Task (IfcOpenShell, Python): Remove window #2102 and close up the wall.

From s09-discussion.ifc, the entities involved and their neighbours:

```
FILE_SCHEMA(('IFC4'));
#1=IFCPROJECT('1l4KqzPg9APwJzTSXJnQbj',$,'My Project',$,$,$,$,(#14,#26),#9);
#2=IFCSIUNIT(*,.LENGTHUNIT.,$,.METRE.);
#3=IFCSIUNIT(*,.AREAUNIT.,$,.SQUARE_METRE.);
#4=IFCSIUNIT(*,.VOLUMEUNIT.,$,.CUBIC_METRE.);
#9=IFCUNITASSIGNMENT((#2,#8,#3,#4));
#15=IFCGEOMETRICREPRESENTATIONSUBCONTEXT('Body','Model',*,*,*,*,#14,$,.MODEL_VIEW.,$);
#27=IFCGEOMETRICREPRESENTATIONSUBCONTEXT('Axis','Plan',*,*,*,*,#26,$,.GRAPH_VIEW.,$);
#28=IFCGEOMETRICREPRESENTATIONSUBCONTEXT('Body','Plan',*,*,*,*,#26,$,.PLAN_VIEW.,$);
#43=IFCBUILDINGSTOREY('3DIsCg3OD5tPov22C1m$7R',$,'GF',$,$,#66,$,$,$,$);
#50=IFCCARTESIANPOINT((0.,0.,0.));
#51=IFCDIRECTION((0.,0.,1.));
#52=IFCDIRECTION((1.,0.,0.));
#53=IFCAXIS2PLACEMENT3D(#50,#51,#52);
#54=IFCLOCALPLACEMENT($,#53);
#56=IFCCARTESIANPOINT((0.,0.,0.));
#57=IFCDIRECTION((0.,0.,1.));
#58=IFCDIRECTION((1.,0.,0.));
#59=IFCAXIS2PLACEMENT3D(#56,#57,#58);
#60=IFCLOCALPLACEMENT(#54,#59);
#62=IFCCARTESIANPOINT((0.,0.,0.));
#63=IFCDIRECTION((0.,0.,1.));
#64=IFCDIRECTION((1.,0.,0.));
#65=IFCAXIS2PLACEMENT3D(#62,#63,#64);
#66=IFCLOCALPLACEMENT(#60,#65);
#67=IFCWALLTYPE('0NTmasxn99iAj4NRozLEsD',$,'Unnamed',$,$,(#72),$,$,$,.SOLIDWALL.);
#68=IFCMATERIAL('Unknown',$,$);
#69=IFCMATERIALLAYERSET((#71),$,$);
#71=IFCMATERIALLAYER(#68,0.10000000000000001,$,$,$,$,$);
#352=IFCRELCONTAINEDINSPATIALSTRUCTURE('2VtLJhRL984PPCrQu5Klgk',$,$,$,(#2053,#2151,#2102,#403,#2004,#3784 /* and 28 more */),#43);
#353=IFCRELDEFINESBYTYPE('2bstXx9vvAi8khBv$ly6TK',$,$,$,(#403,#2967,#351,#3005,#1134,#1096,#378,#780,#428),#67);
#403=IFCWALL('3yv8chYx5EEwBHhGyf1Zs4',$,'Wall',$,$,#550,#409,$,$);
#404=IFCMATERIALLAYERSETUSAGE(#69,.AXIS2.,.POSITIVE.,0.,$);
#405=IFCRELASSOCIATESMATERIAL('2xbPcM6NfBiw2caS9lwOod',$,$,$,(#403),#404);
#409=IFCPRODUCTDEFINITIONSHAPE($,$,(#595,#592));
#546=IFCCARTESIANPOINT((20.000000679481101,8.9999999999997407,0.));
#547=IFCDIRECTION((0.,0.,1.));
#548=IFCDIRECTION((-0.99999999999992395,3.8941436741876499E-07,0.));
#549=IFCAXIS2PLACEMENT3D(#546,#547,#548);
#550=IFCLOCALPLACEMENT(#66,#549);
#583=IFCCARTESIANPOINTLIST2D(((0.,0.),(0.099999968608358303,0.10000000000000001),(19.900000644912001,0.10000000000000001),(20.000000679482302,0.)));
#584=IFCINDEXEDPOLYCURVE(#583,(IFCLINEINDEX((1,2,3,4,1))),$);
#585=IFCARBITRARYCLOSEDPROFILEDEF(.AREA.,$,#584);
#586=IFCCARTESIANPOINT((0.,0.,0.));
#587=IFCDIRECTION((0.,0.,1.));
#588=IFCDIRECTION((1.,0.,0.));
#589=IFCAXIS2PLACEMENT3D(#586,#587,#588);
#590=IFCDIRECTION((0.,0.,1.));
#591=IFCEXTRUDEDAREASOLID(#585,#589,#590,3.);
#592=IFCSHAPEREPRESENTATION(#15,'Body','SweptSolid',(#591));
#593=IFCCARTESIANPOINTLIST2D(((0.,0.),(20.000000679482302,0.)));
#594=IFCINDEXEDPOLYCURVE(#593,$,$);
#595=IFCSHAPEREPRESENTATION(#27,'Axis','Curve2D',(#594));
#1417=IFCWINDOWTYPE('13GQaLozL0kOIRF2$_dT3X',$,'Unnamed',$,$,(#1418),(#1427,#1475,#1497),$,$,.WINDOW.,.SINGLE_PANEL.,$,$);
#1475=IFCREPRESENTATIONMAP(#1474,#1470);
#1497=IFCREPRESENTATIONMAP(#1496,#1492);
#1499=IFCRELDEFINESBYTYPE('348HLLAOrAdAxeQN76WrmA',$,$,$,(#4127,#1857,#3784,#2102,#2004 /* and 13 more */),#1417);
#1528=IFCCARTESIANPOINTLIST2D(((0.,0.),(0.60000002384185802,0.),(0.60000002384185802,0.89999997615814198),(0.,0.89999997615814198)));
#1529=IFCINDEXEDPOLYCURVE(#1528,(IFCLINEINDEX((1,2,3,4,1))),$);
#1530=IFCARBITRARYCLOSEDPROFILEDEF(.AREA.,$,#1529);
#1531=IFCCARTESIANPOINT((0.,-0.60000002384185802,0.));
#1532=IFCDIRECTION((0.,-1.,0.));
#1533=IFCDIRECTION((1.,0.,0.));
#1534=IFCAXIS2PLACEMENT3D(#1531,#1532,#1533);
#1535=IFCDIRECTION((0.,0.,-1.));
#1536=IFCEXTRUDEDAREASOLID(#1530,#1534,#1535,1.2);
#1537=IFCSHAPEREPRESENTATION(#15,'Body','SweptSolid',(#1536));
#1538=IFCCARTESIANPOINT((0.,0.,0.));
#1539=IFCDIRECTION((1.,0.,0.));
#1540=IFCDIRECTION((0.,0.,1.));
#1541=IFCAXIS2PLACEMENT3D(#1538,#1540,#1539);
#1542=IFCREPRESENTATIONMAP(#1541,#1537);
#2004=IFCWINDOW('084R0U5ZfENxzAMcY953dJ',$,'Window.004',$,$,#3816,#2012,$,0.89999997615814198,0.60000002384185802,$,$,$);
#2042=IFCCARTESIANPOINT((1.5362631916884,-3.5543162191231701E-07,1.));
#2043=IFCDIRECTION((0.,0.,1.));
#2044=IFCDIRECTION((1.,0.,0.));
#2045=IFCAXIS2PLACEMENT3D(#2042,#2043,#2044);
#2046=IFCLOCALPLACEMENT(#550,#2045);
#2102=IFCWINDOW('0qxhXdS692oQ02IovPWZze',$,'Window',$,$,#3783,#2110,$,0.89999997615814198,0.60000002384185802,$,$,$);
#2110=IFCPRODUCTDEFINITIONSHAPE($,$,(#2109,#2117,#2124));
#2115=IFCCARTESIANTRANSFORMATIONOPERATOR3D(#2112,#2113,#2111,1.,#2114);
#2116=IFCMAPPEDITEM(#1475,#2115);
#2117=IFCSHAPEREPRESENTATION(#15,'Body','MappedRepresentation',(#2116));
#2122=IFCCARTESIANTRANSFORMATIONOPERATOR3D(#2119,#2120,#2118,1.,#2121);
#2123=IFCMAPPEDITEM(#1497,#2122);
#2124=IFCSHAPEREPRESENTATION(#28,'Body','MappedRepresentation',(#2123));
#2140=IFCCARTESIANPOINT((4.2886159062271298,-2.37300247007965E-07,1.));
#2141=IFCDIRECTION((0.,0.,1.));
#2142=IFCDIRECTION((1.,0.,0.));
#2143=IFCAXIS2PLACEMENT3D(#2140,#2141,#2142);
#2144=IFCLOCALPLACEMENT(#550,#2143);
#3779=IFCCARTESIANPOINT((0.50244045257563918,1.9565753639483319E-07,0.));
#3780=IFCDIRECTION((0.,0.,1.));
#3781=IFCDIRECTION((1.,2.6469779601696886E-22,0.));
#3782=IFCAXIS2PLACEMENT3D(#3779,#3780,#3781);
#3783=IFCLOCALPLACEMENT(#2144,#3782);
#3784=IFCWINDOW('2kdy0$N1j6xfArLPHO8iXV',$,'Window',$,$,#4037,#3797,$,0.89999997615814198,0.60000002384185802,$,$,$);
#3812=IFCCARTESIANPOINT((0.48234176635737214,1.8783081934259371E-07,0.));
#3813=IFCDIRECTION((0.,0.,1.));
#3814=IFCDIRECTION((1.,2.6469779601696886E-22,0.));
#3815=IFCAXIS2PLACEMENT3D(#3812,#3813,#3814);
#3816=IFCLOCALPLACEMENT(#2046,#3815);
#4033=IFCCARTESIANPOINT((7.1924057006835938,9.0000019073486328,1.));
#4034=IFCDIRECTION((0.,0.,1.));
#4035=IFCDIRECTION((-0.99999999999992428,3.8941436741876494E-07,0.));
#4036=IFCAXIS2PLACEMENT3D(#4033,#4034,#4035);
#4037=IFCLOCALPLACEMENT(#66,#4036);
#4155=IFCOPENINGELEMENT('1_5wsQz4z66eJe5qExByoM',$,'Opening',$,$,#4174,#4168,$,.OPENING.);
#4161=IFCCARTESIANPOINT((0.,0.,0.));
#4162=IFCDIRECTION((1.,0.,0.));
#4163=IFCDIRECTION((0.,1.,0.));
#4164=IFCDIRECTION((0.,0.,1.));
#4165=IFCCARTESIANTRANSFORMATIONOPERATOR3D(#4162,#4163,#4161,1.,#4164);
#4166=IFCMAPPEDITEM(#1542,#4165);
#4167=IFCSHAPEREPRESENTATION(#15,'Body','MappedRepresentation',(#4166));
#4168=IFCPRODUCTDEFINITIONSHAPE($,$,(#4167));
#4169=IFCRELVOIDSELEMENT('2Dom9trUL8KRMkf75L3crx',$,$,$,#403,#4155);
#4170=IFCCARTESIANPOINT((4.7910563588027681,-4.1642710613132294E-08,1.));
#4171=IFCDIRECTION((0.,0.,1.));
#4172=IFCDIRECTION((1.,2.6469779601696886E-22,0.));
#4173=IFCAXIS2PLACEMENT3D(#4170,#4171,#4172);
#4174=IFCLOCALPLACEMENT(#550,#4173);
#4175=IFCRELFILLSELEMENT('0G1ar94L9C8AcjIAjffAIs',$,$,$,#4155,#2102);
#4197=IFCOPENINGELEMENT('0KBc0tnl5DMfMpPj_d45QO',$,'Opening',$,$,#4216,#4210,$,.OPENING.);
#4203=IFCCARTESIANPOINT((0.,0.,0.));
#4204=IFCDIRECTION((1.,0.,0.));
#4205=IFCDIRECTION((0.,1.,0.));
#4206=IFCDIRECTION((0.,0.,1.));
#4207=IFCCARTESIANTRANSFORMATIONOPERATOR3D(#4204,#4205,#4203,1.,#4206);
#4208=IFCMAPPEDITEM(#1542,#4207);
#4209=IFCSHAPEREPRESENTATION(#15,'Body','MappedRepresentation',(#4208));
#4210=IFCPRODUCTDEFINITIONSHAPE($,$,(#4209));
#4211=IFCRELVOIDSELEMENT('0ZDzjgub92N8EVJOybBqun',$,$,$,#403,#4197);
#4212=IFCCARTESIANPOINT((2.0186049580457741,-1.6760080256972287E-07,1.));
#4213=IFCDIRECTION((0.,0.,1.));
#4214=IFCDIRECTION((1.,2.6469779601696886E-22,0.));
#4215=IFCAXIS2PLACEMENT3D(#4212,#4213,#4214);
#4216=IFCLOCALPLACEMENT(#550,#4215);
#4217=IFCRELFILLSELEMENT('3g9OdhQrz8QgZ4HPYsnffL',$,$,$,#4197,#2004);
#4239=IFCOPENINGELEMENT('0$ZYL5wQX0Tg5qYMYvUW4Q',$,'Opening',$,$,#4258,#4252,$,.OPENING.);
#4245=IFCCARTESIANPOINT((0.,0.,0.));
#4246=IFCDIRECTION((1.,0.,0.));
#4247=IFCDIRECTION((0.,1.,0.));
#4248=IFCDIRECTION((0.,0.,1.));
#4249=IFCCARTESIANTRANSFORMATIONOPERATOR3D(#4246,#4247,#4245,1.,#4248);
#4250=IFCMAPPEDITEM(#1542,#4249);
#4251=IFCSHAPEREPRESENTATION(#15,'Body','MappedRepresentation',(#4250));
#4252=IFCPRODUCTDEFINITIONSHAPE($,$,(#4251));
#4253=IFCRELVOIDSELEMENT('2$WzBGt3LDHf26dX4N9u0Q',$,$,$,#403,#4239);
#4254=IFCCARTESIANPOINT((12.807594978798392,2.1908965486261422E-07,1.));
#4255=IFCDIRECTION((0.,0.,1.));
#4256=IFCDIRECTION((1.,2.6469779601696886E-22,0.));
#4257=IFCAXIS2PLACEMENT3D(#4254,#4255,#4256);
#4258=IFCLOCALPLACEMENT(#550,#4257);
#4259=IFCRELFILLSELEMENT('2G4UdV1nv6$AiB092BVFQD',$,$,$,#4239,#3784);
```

```python
import ifcopenshell
import ifcopenshell.api.feature
import ifcopenshell.api.root
import ifcopenshell.geom
import ifcopenshell.util.shape

model = ifcopenshell.open("s09-discussion.ifc")
settings = ifcopenshell.geom.settings()


def volume(element):
    """Net volume in cubic metres, openings subtracted."""
    shape = ifcopenshell.geom.create_shape(settings, element)
    return ifcopenshell.util.shape.get_volume(shape.geometry)


window = model.by_guid("0qxhXdS692oQ02IovPWZze")
opening = window.FillsVoids[0].RelatingOpeningElement
wall = opening.VoidsElements[0].RelatingBuildingElement
before = volume(wall)

ifcopenshell.api.root.remove_product(model, product=window)
ifcopenshell.api.feature.remove_feature(model, feature=opening)

after = volume(wall)

print(f"wall volume {before:.3f} -> {after:.3f} m3")

model.write("s09-discussion_edited.ifc")
```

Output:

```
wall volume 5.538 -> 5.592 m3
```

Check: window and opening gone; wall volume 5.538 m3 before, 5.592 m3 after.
